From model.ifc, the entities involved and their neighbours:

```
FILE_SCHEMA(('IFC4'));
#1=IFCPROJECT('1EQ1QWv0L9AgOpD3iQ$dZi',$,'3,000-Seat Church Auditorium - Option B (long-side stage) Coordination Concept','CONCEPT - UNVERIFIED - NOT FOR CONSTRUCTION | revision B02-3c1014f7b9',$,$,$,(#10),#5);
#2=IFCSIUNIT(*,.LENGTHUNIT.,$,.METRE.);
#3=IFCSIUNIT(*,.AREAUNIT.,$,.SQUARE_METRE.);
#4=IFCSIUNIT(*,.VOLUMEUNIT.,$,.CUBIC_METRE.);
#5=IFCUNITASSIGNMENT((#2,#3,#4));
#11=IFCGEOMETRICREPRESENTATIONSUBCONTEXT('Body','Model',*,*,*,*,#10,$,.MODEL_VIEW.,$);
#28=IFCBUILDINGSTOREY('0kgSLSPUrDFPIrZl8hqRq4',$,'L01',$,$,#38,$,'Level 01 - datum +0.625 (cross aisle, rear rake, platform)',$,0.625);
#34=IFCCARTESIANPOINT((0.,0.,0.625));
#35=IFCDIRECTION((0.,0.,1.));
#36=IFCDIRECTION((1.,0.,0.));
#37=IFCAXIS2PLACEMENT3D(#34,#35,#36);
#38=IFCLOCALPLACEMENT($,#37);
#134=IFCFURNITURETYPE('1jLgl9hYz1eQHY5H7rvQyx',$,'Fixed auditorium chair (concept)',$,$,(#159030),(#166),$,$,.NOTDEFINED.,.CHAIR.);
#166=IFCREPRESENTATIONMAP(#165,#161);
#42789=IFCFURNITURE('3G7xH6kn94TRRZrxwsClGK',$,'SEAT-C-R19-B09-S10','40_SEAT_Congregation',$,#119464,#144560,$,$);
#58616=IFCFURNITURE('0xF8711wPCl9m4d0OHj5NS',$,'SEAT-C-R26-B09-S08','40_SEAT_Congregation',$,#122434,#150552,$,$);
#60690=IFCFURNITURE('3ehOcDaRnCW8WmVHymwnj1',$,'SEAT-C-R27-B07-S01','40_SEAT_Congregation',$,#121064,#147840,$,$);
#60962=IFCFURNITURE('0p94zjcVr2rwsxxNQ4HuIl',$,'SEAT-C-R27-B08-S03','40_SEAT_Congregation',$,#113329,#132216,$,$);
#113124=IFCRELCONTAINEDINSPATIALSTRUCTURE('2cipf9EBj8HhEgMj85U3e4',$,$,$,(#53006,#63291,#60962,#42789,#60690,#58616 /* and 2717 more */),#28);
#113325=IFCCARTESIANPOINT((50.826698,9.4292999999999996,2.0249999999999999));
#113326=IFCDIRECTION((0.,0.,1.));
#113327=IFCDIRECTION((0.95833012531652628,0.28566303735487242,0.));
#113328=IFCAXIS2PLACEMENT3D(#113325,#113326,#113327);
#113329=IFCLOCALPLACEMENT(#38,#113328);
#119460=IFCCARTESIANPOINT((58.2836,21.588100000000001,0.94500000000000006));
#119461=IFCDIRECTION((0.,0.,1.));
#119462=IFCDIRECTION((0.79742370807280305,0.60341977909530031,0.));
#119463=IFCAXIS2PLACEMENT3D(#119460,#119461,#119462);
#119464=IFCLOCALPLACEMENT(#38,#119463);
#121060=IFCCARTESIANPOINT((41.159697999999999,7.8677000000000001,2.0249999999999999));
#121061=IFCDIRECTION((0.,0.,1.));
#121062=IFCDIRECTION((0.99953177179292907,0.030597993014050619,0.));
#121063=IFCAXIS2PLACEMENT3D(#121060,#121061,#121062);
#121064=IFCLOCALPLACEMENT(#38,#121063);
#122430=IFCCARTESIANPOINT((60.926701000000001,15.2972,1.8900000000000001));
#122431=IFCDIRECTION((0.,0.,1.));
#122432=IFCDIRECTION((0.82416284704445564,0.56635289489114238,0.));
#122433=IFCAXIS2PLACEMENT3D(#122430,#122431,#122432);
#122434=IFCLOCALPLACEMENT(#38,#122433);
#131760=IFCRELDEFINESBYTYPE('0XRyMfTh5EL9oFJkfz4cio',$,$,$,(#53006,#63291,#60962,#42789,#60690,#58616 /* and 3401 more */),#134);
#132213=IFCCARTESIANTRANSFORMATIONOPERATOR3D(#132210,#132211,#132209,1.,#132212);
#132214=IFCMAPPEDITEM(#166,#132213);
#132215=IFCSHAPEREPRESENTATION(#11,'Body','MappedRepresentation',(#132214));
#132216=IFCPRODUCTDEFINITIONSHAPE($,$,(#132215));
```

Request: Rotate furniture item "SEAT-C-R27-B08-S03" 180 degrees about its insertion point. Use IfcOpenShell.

```python
import ifcopenshell
import ifcopenshell.api.geometry
import ifcopenshell.util.placement

model = ifcopenshell.open("model.ifc")

item = model.by_guid("0p94zjcVr2rwsxxNQ4HuIl")
matrix = ifcopenshell.util.placement.get_local_placement(item.ObjectPlacement)
matrix = matrix @ ifcopenshell.util.placement.rotation(180, "Z")
ifcopenshell.api.geometry.edit_object_placement(model, product=item, matrix=matrix, is_si=False)

print(ifcopenshell.util.placement.get_local_placement(item.ObjectPlacement).round(3) + 0.0)

model.write("model_updated.ifc")
```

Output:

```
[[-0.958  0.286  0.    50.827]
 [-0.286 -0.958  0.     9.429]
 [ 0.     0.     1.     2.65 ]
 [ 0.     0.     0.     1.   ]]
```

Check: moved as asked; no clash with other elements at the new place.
